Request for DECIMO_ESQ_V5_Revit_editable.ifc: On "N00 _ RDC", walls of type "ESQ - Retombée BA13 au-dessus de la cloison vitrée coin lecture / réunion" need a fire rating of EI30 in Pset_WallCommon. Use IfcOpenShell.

First a look at what the model holds.

```python
import ifcopenshell
import ifcopenshell.util.element

model = ifcopenshell.open("DECIMO_ESQ_V5_Revit_editable.ifc")
print(model.schema)
storey = next(s for s in model.by_type("IfcBuildingStorey") if s.Name == "N00 _ RDC")
walls = [e for e in ifcopenshell.util.element.get_decomposition(storey) if e.is_a("IfcWall")]
seen = {}
for e in walls:
    element_type = ifcopenshell.util.element.get_type(e)
    key = (element_type.Name if element_type != e and element_type else None, ifcopenshell.util.element.get_pset(e, "Pset_WallCommon", "FireRating"))
    seen[key] = seen.get(key, 0) + 1
for (name, value), count in sorted(seen.items(), key=str):
    print(count, "x", name, "|", value)
```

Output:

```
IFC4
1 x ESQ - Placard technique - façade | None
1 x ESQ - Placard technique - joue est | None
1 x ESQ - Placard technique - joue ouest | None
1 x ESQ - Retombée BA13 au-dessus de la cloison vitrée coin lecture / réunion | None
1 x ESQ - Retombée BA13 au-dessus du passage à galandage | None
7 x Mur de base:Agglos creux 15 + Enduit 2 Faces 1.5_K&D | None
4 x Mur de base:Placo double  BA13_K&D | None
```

```python
import ifcopenshell
import ifcopenshell.api.pset
import ifcopenshell.util.element

model = ifcopenshell.open("DECIMO_ESQ_V5_Revit_editable.ifc")

storey = next(s for s in model.by_type("IfcBuildingStorey") if s.Name == "N00 _ RDC")
walls = [e for e in ifcopenshell.util.element.get_decomposition(storey) if e.is_a("IfcWall")]

count = 0
for e in walls:
    element_type = ifcopenshell.util.element.get_type(e)
    if element_type in (None, e) or element_type.Name != "ESQ - Retombée BA13 au-dessus de la cloison vitrée coin lecture / réunion":
        continue
    # add_pset returns the element's existing set when there is one.
    pset = ifcopenshell.api.pset.add_pset(model, product=e, name="Pset_WallCommon")
    ifcopenshell.api.pset.edit_pset(model, pset=pset, properties={"FireRating": "EI30"})
    count += 1

print(count, "walls updated")

model.write("DECIMO_ESQ_V5_Revit_editable_edited.ifc")
```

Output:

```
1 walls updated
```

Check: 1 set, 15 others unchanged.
